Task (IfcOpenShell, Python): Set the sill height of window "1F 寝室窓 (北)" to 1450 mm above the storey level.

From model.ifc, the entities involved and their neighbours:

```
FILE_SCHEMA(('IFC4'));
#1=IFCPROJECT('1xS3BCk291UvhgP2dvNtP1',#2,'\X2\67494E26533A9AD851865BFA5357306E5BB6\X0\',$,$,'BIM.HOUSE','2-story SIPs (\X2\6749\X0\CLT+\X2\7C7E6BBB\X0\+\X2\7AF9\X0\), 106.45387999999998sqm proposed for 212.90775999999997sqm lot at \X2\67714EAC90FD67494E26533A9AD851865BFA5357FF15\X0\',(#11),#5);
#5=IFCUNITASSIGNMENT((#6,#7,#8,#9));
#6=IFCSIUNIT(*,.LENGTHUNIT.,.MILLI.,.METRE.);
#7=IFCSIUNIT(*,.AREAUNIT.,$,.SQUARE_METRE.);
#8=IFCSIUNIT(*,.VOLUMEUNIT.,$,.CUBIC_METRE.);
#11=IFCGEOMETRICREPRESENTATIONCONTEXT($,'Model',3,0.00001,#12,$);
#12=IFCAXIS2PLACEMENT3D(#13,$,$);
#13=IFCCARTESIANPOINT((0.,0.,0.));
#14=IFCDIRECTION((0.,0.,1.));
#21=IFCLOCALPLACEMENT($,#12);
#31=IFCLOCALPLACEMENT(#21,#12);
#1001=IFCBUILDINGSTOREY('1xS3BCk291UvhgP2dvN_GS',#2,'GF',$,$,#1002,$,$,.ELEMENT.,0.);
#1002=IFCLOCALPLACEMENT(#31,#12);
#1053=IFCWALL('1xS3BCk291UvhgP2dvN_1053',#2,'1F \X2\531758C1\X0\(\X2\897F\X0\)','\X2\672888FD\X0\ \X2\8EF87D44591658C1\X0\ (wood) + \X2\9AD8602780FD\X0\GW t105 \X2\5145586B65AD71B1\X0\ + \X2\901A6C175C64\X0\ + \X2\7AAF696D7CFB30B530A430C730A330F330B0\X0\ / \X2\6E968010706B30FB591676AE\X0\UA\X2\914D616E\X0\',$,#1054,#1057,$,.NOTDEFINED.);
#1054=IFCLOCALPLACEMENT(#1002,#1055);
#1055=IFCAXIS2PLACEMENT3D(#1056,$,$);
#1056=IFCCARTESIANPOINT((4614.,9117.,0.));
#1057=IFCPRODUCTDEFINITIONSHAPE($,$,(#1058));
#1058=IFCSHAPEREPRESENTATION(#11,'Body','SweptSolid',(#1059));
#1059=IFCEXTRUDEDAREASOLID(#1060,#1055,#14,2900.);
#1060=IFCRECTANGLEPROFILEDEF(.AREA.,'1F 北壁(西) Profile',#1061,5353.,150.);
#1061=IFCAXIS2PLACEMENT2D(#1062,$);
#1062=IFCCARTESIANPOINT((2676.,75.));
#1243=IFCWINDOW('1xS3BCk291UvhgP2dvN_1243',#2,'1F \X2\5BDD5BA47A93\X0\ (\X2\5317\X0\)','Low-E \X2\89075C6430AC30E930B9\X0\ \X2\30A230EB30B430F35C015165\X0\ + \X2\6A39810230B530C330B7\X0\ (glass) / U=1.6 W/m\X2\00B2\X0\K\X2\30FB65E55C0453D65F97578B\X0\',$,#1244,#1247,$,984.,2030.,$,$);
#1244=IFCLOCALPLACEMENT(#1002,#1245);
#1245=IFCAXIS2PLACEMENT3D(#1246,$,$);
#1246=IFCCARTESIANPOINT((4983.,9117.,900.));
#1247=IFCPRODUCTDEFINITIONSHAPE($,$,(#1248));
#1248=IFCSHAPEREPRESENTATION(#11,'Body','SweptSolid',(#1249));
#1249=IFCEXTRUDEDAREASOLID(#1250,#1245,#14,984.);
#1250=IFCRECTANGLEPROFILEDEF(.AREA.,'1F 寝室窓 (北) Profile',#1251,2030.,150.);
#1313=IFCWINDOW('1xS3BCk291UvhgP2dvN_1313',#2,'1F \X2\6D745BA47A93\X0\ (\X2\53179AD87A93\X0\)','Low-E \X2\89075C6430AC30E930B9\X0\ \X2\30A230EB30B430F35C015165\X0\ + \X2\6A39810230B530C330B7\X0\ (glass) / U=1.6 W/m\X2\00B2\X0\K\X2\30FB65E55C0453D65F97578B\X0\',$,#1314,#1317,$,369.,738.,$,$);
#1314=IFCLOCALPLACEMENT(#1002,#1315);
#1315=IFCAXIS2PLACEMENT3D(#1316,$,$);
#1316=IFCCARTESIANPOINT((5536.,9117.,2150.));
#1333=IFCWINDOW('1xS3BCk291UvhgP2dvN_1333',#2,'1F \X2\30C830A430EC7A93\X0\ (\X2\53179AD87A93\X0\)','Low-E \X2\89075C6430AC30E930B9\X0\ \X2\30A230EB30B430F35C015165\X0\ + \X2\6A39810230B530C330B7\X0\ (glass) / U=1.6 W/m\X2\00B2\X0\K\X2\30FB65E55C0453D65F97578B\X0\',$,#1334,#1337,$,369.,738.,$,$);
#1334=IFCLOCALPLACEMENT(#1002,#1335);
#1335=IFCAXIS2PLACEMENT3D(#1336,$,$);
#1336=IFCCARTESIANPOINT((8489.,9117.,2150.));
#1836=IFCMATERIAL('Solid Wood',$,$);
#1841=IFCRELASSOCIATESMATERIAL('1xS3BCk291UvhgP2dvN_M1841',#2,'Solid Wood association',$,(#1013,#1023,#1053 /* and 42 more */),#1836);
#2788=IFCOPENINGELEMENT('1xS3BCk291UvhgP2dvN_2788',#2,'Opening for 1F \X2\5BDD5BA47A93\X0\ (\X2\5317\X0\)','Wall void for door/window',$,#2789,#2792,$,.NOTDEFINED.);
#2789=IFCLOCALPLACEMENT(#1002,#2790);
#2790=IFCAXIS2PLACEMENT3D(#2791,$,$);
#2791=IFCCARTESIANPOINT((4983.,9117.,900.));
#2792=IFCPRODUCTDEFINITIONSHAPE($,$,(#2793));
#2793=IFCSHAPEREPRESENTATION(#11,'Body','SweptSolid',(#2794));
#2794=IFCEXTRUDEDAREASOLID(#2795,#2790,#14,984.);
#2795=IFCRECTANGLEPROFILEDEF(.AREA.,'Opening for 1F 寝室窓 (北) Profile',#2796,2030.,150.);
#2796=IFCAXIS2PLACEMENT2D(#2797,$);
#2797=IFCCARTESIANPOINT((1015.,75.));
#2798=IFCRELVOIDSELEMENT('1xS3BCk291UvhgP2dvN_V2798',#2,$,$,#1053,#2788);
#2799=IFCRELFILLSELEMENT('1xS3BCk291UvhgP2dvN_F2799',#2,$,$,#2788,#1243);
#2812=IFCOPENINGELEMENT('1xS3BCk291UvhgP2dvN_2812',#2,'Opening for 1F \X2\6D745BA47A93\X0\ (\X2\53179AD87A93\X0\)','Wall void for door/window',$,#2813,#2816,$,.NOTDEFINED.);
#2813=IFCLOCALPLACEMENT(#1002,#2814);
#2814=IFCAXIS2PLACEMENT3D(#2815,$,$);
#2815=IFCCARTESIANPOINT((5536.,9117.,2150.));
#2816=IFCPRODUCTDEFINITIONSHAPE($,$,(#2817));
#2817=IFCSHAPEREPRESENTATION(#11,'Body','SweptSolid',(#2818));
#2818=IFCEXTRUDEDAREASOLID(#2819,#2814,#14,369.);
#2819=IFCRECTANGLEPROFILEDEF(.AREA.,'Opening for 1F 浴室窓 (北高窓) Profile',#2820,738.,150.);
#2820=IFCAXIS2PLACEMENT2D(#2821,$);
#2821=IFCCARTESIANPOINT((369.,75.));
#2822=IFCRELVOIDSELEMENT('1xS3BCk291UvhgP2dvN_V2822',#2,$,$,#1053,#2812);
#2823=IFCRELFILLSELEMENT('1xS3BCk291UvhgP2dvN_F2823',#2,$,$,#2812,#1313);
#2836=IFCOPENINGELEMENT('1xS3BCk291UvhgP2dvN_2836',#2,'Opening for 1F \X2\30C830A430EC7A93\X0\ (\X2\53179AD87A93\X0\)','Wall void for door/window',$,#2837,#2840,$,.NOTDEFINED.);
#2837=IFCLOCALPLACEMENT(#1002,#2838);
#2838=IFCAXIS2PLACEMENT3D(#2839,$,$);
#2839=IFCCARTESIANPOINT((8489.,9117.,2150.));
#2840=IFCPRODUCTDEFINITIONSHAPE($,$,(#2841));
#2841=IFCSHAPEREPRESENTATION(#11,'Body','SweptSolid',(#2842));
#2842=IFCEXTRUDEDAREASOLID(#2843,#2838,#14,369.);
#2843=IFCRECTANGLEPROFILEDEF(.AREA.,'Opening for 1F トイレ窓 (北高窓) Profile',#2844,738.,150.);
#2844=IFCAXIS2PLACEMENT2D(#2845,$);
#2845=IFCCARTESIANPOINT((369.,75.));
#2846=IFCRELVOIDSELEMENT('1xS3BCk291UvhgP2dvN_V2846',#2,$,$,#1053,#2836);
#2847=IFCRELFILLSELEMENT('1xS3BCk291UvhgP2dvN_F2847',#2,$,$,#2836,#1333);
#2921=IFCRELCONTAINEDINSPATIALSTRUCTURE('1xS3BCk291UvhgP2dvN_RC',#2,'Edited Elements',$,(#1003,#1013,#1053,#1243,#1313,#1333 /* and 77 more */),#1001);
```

```python
import numpy as np
import ifcopenshell
import ifcopenshell.api.geometry
import ifcopenshell.geom
import ifcopenshell.util.element
import ifcopenshell.util.placement
import ifcopenshell.util.shape
import ifcopenshell.util.unit

model = ifcopenshell.open("model.ifc")
unit_scale = ifcopenshell.util.unit.calculate_unit_scale(model)

window = model.by_id(1243)
opening = window.FillsVoids[0].RelatingOpeningElement
storey = ifcopenshell.util.element.get_container(window, ifc_class="IfcBuildingStorey")
level = ifcopenshell.util.placement.get_local_placement(storey.ObjectPlacement)[2, 3]

# The opening's origin need not be at the sill, so measure its lowest point.
shape = ifcopenshell.geom.create_shape(ifcopenshell.geom.settings(), opening)
bottom = ifcopenshell.util.shape.get_shape_bottom_elevation(shape, shape.geometry) / unit_scale
dz = level + 1.45 / unit_scale - bottom

shift = np.array([0.0, 0.0, dz])
# The window is not placed relative to its opening, so move both.
for product in (opening, window):
    matrix = ifcopenshell.util.placement.get_local_placement(product.ObjectPlacement)
    matrix[:3, 3] += shift
    ifcopenshell.api.geometry.edit_object_placement(model, product=product, matrix=matrix, is_si=False)

print(f"moved by {dz * unit_scale:+.3f} m")

model.write("model_v2.ifc")
```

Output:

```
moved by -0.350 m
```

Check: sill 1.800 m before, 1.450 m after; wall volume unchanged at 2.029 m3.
